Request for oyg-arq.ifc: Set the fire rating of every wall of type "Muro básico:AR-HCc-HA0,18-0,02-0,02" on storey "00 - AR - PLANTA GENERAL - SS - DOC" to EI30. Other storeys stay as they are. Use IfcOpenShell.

First a look at what the model holds.

```python
import ifcopenshell
import ifcopenshell.util.element

model = ifcopenshell.open("oyg-arq.ifc")
print(model.schema)
storey = next(s for s in model.by_type("IfcBuildingStorey") if s.Name == "00 - AR - PLANTA GENERAL - SS - DOC")
walls = [e for e in ifcopenshell.util.element.get_decomposition(storey) if e.is_a("IfcWall")]
seen = {}
for e in walls:
    element_type = ifcopenshell.util.element.get_type(e)
    key = (element_type.Name if element_type != e and element_type else None, ifcopenshell.util.element.get_pset(e, "Pset_WallCommon", "FireRating"))
    seen[key] = seen.get(key, 0) + 1
for (name, value), count in sorted(seen.items(), key=str):
    print(count, "x", name, "|", value)
```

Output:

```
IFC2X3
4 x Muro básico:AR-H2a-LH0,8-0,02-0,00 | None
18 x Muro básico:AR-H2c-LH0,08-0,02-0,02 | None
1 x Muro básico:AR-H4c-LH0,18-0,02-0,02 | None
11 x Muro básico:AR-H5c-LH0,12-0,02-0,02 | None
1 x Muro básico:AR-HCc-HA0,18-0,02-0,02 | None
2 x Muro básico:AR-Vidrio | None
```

```python
import ifcopenshell
import ifcopenshell.api.pset
import ifcopenshell.util.element

model = ifcopenshell.open("oyg-arq.ifc")

storey = next(s for s in model.by_type("IfcBuildingStorey") if s.Name == "00 - AR - PLANTA GENERAL - SS - DOC")
walls = [e for e in ifcopenshell.util.element.get_decomposition(storey) if e.is_a("IfcWall")]

count = 0
for e in walls:
    element_type = ifcopenshell.util.element.get_type(e)
    if element_type in (None, e) or element_type.Name != "Muro básico:AR-HCc-HA0,18-0,02-0,02":
        continue
    # add_pset returns the element's existing set when there is one.
    pset = ifcopenshell.api.pset.add_pset(model, product=e, name="Pset_WallCommon")
    ifcopenshell.api.pset.edit_pset(model, pset=pset, properties={"FireRating": "EI30"})
    count += 1

print(count, "walls updated")

model.write("oyg-arq_edited.ifc")
```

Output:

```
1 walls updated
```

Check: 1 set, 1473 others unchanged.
